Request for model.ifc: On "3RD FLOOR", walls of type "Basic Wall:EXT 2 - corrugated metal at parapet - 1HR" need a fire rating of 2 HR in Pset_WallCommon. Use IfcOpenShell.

First a look at what the model holds.

```python
import ifcopenshell
import ifcopenshell.util.element

model = ifcopenshell.open("model.ifc")
print(model.schema)
storey = next(s for s in model.by_type("IfcBuildingStorey") if s.Name == "3RD FLOOR")
walls = [e for e in ifcopenshell.util.element.get_decomposition(storey) if e.is_a("IfcWall")]
seen = {}
for e in walls:
    element_type = ifcopenshell.util.element.get_type(e)
    key = (element_type.Name if element_type != e and element_type else None, ifcopenshell.util.element.get_pset(e, "Pset_WallCommon", "FireRating"))
    seen[key] = seen.get(key, 0) + 1
for (name, value), count in sorted(seen.items(), key=str):
    print(count, "x", name, "|", value)
```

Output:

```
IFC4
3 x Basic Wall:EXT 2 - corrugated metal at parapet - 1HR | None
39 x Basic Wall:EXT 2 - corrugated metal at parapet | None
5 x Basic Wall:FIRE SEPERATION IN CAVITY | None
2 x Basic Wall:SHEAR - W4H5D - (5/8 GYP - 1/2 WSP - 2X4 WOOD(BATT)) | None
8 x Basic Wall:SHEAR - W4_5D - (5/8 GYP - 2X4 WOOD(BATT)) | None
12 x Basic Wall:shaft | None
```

```python
import ifcopenshell
import ifcopenshell.api.pset
import ifcopenshell.util.element

model = ifcopenshell.open("model.ifc")

storey = next(s for s in model.by_type("IfcBuildingStorey") if s.Name == "3RD FLOOR")
walls = [e for e in ifcopenshell.util.element.get_decomposition(storey) if e.is_a("IfcWall")]

count = 0
for e in walls:
    element_type = ifcopenshell.util.element.get_type(e)
    if element_type in (None, e) or element_type.Name != "Basic Wall:EXT 2 - corrugated metal at parapet - 1HR":
        continue
    # add_pset returns the element's existing set when there is one.
    pset = ifcopenshell.api.pset.add_pset(model, product=e, name="Pset_WallCommon")
    ifcopenshell.api.pset.edit_pset(model, pset=pset, properties={"FireRating": "2 HR"})
    count += 1

print(count, "walls updated")

model.write("model_rev.ifc")
```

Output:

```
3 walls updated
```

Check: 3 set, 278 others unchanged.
